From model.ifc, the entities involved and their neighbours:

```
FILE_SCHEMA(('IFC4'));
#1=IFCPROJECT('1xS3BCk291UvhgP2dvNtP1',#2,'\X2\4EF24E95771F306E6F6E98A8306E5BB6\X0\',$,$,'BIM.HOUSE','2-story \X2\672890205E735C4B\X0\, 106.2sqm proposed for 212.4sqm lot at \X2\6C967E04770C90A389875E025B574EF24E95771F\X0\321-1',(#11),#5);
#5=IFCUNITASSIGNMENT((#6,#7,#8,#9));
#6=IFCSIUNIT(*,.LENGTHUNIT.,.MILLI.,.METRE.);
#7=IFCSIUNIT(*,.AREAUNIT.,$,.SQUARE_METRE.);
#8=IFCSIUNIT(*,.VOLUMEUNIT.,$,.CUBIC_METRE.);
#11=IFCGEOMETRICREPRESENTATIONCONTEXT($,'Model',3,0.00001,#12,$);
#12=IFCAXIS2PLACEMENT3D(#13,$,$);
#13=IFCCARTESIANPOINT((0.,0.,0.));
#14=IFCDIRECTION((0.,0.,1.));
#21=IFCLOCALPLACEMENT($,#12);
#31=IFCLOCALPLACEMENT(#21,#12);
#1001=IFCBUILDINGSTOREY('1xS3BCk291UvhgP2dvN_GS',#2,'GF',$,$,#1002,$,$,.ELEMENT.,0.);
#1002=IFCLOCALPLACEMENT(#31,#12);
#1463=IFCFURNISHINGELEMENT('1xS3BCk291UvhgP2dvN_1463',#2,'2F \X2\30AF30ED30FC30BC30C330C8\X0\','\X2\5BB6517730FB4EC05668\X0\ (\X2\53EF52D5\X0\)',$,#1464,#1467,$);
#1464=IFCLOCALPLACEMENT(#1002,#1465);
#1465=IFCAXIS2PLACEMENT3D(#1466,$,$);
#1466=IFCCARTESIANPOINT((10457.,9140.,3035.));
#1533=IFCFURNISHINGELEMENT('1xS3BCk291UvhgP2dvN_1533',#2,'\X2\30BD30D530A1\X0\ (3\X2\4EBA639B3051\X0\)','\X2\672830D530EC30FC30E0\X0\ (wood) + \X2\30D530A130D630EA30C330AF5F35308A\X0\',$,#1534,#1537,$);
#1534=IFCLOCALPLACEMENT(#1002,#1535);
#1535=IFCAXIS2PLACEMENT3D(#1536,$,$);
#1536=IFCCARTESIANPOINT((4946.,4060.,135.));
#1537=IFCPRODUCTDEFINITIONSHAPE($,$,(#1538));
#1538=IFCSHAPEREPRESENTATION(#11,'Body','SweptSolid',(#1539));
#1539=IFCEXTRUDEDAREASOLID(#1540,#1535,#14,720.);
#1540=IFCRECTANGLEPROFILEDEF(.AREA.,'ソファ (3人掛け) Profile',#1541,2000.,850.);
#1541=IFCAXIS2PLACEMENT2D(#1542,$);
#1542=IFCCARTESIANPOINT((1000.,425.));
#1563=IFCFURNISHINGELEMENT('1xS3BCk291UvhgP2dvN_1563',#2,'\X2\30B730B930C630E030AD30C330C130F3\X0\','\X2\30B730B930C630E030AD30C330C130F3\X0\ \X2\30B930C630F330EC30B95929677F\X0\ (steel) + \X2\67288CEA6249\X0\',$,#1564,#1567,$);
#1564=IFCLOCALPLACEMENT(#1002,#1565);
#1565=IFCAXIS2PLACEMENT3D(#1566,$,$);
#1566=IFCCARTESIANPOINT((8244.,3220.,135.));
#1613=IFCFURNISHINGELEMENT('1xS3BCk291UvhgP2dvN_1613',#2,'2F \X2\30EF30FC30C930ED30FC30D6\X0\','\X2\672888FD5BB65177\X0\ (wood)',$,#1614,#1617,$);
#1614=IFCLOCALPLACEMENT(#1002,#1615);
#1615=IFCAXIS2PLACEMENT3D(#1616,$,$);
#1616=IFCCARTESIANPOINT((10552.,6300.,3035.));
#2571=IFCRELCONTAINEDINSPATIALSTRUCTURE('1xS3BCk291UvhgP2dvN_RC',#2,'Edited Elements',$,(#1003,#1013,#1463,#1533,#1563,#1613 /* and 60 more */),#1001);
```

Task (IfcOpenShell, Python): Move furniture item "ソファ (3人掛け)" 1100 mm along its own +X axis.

```python
import ifcopenshell
import ifcopenshell.api.geometry
import ifcopenshell.util.placement

model = ifcopenshell.open("model.ifc")

item = model.by_guid("1xS3BCk291UvhgP2dvN_1533")
matrix = ifcopenshell.util.placement.get_local_placement(item.ObjectPlacement)
matrix[:3, 3] += matrix[:3, 0] * 1100.0
ifcopenshell.api.geometry.edit_object_placement(model, product=item, matrix=matrix, is_si=False)

print(ifcopenshell.util.placement.get_local_placement(item.ObjectPlacement).round(3) + 0.0)

model.write("model-out.ifc")
```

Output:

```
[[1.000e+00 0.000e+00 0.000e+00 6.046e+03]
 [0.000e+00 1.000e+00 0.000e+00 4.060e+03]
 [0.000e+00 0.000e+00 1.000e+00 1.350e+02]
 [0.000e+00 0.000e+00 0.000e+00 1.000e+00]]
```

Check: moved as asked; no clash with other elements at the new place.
